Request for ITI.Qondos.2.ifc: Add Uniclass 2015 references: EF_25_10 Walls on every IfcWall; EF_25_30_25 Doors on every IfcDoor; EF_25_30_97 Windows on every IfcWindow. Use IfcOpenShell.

First a look at what the model holds.

```python
import ifcopenshell

model = ifcopenshell.open("ITI.Qondos.2.ifc")
print(model.schema)
print("classifications:", [c.Name for c in model.by_type("IfcClassification")])
for ifc_class in ("IfcDoor", "IfcRoof", "IfcStair", "IfcWall", "IfcWindow"):
    print(ifc_class, len(model.by_type(ifc_class)))
```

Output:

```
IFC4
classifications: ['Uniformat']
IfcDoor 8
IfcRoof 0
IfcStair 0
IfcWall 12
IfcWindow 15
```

```python
import ifcopenshell
import ifcopenshell.api.classification

model = ifcopenshell.open("ITI.Qondos.2.ifc")

system = ifcopenshell.api.classification.add_classification(model, classification="Uniclass 2015")

codes = {
    "IfcWall": ("EF_25_10", "Walls"),
    "IfcDoor": ("EF_25_30_25", "Doors"),
    "IfcWindow": ("EF_25_30_97", "Windows"),
}
for ifc_class, (code, name) in codes.items():
    products = model.by_type(ifc_class)
    ifcopenshell.api.classification.add_reference(
        model, products=products, classification=system, identification=code, name=name
    )
    print(code, len(products))

model.write("ITI.Qondos.2_v2.ifc")
```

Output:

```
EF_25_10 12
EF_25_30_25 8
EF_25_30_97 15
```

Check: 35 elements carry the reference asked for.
